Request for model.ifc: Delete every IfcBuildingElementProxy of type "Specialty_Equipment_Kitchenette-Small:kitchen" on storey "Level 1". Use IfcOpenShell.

First a look at what the model holds.

```python
import ifcopenshell
import ifcopenshell.util.element

model = ifcopenshell.open("model.ifc")
print(model.schema)
storey = next(s for s in model.by_type("IfcBuildingStorey") if s.Name == "Level 1")
proxies = [e for e in ifcopenshell.util.element.get_decomposition(storey) if e.is_a("IfcBuildingElementProxy")]
seen = {}
for e in proxies:
    element_type = ifcopenshell.util.element.get_type(e)
    name = element_type.Name if element_type not in (None, e) else None
    seen[name] = seen.get(name, 0) + 1
for name, count in sorted(seen.items(), key=str):
    print(count, "x", name)
```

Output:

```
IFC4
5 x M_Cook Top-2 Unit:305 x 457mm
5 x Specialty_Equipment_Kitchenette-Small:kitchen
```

```python
import ifcopenshell
import ifcopenshell.api.root
import ifcopenshell.util.element

model = ifcopenshell.open("model.ifc")

storey = next(s for s in model.by_type("IfcBuildingStorey") if s.Name == "Level 1")
proxies = [e for e in ifcopenshell.util.element.get_decomposition(storey) if e.is_a("IfcBuildingElementProxy")]
targets = [e for e in proxies if (t := ifcopenshell.util.element.get_type(e)) not in (None, e) and t.Name == "Specialty_Equipment_Kitchenette-Small:kitchen"]

for e in targets:
    ifcopenshell.api.root.remove_product(model, product=e)
print(len(targets), "removed")

model.write("model-out.ifc")
```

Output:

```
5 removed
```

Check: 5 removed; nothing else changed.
